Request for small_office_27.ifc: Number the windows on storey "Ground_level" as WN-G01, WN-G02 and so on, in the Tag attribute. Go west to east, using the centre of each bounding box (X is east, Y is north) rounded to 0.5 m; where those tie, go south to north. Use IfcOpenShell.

First a look at what the model holds.

```python
import ifcopenshell
import ifcopenshell.util.element
import ifcopenshell.util.placement

model = ifcopenshell.open("small_office_27.ifc")
print(model.schema)
storey = next(s for s in model.by_type("IfcBuildingStorey") if s.Name == "Ground_level")
windows = [e for e in ifcopenshell.util.element.get_decomposition(storey) if e.is_a("IfcWindow")]
for e in sorted(windows, key=lambda e: e.id()):
    origin = ifcopenshell.util.placement.get_local_placement(e.ObjectPlacement)[:3, 3]
    print(e.id(), e.Tag, e.Name, origin.round(2) + 0.0, sep=" | ")
```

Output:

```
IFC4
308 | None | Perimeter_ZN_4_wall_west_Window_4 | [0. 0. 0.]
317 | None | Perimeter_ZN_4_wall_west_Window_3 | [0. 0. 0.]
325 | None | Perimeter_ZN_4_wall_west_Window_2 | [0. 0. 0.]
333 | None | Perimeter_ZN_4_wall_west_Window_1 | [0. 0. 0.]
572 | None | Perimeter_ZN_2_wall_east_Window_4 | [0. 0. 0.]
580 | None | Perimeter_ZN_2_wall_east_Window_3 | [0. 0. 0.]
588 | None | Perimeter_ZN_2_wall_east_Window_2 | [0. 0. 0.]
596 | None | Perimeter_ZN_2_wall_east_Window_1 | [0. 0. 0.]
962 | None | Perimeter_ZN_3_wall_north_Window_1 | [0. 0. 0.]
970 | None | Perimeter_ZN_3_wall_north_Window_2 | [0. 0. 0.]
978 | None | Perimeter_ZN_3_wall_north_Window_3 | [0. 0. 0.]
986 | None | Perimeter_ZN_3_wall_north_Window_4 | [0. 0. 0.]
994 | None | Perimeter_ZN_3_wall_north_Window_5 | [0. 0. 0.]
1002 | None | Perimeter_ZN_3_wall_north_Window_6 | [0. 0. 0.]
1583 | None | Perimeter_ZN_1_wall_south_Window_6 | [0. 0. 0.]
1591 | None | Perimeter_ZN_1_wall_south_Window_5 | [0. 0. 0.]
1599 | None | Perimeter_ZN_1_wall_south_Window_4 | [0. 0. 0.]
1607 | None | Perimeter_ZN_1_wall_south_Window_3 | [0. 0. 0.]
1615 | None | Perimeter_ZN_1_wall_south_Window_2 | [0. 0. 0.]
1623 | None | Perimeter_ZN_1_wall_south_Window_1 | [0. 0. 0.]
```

```python
import ifcopenshell
import ifcopenshell.geom
import ifcopenshell.util.element
import ifcopenshell.util.shape

model = ifcopenshell.open("small_office_27.ifc")
settings = ifcopenshell.geom.settings()
settings.set("use-world-coords", True)


def centre(element):
    shape = ifcopenshell.geom.create_shape(settings, element)
    return ifcopenshell.util.shape.get_bbox_centroid(shape.geometry)


storey = next(s for s in model.by_type("IfcBuildingStorey") if s.Name == "Ground_level")
windows = [e for e in ifcopenshell.util.element.get_decomposition(storey) if e.is_a("IfcWindow")]

# Insertion points can sit at a corner or the storey origin, so sort by the geometry (in metres).
centres = {e: centre(e) for e in windows}
windows.sort(key=lambda e: (round(centres[e][0] / 0.5), centres[e][1]))

for i, e in enumerate(windows, start=1):
    number = f"WN-G{i:02d}"
    e.Tag = number
    print(e.id(), number)

model.write("small_office_27_edited.ifc")
```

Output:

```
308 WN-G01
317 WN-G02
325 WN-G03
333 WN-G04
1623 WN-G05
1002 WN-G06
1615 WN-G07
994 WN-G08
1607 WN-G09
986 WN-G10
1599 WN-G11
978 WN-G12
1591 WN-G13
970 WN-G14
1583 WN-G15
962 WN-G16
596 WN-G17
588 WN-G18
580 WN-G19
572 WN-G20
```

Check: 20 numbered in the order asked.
